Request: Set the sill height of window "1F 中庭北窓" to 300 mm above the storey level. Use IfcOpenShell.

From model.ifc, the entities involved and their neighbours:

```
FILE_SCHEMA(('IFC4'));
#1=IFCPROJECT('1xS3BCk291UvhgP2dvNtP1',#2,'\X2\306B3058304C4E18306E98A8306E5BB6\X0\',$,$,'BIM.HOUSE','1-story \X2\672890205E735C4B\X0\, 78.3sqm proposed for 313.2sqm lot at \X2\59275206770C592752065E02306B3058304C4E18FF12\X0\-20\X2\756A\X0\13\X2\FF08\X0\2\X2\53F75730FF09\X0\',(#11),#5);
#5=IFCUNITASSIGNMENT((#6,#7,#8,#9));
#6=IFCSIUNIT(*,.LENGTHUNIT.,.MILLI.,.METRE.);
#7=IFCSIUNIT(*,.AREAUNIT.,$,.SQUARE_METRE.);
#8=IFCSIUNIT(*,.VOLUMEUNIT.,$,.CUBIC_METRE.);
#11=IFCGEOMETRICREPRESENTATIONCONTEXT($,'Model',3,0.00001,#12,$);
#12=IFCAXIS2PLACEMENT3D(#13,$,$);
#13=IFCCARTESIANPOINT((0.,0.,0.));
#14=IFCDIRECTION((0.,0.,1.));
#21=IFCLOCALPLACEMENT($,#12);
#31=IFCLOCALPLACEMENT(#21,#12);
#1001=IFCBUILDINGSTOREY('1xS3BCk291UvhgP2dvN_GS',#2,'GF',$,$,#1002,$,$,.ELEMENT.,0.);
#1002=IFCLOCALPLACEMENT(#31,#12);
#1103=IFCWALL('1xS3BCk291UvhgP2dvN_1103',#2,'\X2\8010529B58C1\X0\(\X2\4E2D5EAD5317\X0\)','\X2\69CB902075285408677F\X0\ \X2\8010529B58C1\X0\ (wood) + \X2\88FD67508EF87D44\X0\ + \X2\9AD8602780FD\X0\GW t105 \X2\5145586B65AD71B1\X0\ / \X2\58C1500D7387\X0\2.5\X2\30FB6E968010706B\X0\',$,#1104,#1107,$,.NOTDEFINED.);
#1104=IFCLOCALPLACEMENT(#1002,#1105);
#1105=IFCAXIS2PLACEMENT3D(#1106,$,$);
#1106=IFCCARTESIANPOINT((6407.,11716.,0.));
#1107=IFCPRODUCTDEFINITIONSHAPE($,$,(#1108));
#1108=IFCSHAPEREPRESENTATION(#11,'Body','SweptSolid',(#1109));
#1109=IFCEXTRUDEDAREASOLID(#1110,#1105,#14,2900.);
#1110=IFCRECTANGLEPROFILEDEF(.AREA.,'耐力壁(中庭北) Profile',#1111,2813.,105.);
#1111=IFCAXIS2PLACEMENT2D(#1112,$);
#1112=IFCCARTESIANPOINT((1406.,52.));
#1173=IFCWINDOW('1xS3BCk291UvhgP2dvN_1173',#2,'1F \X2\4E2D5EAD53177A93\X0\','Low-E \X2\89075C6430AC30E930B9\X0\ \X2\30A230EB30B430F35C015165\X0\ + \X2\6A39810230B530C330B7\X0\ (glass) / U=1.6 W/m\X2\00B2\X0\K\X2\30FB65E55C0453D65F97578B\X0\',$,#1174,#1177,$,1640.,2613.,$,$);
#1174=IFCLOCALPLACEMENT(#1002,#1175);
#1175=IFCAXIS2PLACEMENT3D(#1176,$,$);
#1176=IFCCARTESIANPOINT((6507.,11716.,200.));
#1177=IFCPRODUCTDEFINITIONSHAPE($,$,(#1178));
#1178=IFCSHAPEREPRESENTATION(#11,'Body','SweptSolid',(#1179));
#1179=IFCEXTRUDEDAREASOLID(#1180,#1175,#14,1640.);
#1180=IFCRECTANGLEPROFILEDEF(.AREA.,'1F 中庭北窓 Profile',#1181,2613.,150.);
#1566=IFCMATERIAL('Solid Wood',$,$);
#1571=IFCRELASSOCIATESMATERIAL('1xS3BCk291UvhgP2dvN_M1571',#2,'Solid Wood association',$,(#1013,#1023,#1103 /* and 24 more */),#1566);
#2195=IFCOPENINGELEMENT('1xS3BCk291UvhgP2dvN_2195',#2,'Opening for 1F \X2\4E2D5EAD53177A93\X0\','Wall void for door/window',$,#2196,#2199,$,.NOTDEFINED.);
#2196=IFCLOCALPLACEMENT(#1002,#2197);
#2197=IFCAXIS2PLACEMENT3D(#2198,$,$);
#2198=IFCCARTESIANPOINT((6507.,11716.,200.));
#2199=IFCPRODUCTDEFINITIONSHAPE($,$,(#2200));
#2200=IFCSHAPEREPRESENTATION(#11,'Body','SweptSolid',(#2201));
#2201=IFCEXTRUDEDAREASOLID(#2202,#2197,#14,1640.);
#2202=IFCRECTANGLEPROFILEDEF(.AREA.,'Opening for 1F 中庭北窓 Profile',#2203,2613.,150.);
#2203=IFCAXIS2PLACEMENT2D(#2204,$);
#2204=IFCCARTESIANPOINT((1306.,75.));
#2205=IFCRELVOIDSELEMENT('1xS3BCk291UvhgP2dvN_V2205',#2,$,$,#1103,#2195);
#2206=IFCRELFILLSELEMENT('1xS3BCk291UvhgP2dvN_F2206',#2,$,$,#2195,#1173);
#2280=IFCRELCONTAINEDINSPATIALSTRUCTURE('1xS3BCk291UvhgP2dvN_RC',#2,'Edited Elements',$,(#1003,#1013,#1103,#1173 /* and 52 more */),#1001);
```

```python
import numpy as np
import ifcopenshell
import ifcopenshell.api.geometry
import ifcopenshell.geom
import ifcopenshell.util.element
import ifcopenshell.util.placement
import ifcopenshell.util.shape
import ifcopenshell.util.unit

model = ifcopenshell.open("model.ifc")
unit_scale = ifcopenshell.util.unit.calculate_unit_scale(model)

window = model.by_guid("1xS3BCk291UvhgP2dvN_1173")
opening = window.FillsVoids[0].RelatingOpeningElement
storey = ifcopenshell.util.element.get_container(window, ifc_class="IfcBuildingStorey")
level = ifcopenshell.util.placement.get_local_placement(storey.ObjectPlacement)[2, 3]

# The opening's origin need not be at the sill, so measure its lowest point.
shape = ifcopenshell.geom.create_shape(ifcopenshell.geom.settings(), opening)
bottom = ifcopenshell.util.shape.get_shape_bottom_elevation(shape, shape.geometry) / unit_scale
dz = level + 300.0 - bottom

shift = np.array([0.0, 0.0, dz])
# The window is not placed relative to its opening, so move both.
for product in (opening, window):
    matrix = ifcopenshell.util.placement.get_local_placement(product.ObjectPlacement)
    matrix[:3, 3] += shift
    ifcopenshell.api.geometry.edit_object_placement(model, product=product, matrix=matrix, is_si=False)

print(f"moved by {dz * unit_scale:+.3f} m")

model.write("model_updated.ifc")
```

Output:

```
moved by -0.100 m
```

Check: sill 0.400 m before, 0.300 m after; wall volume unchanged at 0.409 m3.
